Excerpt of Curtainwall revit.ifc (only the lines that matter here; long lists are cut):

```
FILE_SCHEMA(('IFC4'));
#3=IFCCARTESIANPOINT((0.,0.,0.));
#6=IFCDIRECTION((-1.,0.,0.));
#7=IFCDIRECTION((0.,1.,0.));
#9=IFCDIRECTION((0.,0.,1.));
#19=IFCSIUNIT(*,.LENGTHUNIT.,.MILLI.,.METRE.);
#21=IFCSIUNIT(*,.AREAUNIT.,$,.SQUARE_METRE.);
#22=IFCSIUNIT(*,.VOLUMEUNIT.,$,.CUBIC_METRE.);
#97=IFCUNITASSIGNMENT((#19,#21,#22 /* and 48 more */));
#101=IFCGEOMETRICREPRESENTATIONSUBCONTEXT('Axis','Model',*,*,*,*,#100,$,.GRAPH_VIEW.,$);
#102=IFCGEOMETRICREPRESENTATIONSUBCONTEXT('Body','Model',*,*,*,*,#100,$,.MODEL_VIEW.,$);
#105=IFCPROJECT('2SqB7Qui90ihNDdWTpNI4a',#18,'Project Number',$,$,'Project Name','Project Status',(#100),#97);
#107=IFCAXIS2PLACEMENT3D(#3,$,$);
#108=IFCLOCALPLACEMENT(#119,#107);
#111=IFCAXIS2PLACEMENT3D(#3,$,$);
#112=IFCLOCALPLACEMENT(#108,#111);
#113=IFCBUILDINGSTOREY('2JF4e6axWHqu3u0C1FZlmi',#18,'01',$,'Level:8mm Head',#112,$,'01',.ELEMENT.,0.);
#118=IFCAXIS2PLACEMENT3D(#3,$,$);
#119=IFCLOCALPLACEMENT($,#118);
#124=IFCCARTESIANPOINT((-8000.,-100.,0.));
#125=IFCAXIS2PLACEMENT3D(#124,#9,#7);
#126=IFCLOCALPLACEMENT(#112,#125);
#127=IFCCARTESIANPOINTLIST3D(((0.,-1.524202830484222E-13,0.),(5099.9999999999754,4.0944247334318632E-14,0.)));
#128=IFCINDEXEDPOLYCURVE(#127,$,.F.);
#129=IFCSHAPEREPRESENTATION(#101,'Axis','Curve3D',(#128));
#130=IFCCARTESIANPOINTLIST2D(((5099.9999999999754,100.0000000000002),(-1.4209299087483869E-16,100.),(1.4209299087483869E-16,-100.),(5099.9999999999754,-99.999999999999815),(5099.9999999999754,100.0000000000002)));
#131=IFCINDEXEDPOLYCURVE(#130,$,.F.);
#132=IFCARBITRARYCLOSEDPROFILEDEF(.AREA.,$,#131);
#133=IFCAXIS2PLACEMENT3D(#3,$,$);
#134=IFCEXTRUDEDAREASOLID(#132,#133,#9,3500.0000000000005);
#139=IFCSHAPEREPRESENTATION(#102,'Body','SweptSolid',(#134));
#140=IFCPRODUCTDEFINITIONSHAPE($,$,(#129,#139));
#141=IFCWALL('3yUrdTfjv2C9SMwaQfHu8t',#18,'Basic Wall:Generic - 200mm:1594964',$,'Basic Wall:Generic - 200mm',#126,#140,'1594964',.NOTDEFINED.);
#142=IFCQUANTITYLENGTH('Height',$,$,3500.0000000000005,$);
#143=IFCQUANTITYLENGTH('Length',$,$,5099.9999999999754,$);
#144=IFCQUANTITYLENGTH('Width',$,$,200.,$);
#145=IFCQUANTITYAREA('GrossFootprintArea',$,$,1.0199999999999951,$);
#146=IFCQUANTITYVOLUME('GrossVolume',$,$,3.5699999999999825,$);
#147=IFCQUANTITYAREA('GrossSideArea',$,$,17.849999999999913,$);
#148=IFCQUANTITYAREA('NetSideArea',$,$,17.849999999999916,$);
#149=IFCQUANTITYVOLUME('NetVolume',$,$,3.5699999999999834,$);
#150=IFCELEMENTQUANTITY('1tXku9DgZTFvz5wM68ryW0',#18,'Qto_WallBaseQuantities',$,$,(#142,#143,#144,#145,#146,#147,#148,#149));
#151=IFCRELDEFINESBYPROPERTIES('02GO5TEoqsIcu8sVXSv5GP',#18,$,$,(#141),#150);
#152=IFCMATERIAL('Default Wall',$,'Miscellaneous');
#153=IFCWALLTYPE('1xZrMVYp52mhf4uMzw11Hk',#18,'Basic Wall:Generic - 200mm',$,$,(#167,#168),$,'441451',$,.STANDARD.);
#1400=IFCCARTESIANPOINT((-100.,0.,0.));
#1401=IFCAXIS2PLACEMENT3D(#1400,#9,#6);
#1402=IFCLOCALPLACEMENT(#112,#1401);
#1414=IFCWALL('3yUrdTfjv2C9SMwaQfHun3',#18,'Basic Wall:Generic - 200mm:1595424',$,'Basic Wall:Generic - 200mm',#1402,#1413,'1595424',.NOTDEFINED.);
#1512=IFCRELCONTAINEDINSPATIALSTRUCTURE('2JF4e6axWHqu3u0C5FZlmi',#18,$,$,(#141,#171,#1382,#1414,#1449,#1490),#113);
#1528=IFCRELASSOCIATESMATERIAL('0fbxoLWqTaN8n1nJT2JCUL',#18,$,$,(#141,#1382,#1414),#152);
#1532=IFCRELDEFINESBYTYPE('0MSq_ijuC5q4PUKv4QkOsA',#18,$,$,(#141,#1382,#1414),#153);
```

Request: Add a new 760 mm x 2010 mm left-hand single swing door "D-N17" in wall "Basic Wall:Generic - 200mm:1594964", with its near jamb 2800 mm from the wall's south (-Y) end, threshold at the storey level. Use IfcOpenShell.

```python
import numpy as np
import ifcopenshell
import ifcopenshell.api.feature
import ifcopenshell.api.geometry
import ifcopenshell.api.pset
import ifcopenshell.api.root
import ifcopenshell.api.spatial
import ifcopenshell.geom
import ifcopenshell.util.element
import ifcopenshell.util.placement
import ifcopenshell.util.representation
import ifcopenshell.util.shape
import ifcopenshell.util.unit

model = ifcopenshell.open("Curtainwall revit.ifc")
unit_scale = ifcopenshell.util.unit.calculate_unit_scale(model)
area_scale = ifcopenshell.util.unit.calculate_unit_scale(model, "AREAUNIT")
volume_scale = ifcopenshell.util.unit.calculate_unit_scale(model, "VOLUMEUNIT")
settings = ifcopenshell.geom.settings()


def volume(element):
    """Net volume in cubic metres, openings subtracted."""
    shape = ifcopenshell.geom.create_shape(settings, element)
    return ifcopenshell.util.shape.get_volume(shape.geometry)


wall = model.by_id(141)
storey = ifcopenshell.util.element.get_container(wall, ifc_class="IfcBuildingStorey")
context = ifcopenshell.util.representation.get_context(model, "Model", "Body", "MODEL_VIEW")
before = volume(wall)

width, height, from_end, sill = 0.76, 2.01, 2.8, 0.0  # metres

# The wall runs along its own X axis, and the end named is its -X end.
wall_shape = ifcopenshell.geom.create_shape(settings, wall)
x, y, z = ifcopenshell.util.shape.get_vertices(wall_shape.geometry).T
start = x.min() + from_end
face, thickness = float(y.min()), float(y.max() - y.min())
wall_matrix = ifcopenshell.util.placement.get_local_placement(wall.ObjectPlacement)
level = ifcopenshell.util.placement.get_local_placement(storey.ObjectPlacement)[2, 3]


def in_wall(x, y):
    """Placement at x, y metres in the wall's axes, at sill height."""
    matrix = wall_matrix.copy()
    matrix[:, 3] = wall_matrix @ np.array([x / unit_scale, y / unit_scale, 0.0, 1.0])
    matrix[2, 3] = level + sill / unit_scale
    return matrix


# Opening: a box that overshoots both wall faces by 50 mm.
opening = ifcopenshell.api.root.create_entity(model, ifc_class="IfcOpeningElement", predefined_type="OPENING")
box = ifcopenshell.api.geometry.add_wall_representation(
    model, context=context, length=width, height=height, thickness=thickness + 0.1
)
ifcopenshell.api.geometry.assign_representation(model, product=opening, representation=box)
ifcopenshell.api.geometry.edit_object_placement(model, product=opening, matrix=in_wall(start, face - 0.05), is_si=False)
ifcopenshell.api.feature.add_feature(model, feature=opening, element=wall)

door = ifcopenshell.api.root.create_entity(model, ifc_class="IfcDoor", name="D-N17", predefined_type="DOOR")
door.OverallWidth, door.OverallHeight = width / unit_scale, height / unit_scale
door.OperationType = "SINGLE_SWING_LEFT"
body = ifcopenshell.api.geometry.add_door_representation(
    model,
    context=context,
    overall_width=door.OverallWidth,
    overall_height=door.OverallHeight,
    operation_type="SINGLE_SWING_LEFT",
    lining_properties={"LiningDepth": thickness / unit_scale, "ThresholdDepth": thickness / unit_scale},
)
ifcopenshell.api.geometry.assign_representation(model, product=door, representation=body)
ifcopenshell.api.spatial.assign_container(model, products=[door], relating_structure=storey)
ifcopenshell.api.feature.add_filling(model, opening=opening, element=door)

# The lining spans the wall, so the door starts at the wall face.
ifcopenshell.api.geometry.edit_object_placement(model, product=door, matrix=in_wall(start, face), is_si=False)

after = volume(wall)

# Update the wall's stored quantities.
qto = model.by_id(ifcopenshell.util.element.get_pset(wall, "Qto_WallBaseQuantities", should_inherit=False)["id"])
ifcopenshell.api.pset.edit_qto(model, qto=qto, properties={
    "NetSideArea": after / thickness / area_scale,
    "NetVolume": after / volume_scale,
})

print(f"wall volume {before:.3f} -> {after:.3f} m3")

model.write("Curtainwall revit_rev.ifc")
```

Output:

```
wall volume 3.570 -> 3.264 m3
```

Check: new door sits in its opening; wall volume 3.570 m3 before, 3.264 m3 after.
